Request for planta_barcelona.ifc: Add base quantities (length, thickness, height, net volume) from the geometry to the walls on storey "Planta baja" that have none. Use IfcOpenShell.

First a look at what the model holds.

```python
import ifcopenshell
import ifcopenshell.util.element
import ifcopenshell.util.unit

model = ifcopenshell.open("planta_barcelona.ifc")
print(model.schema)
for unit_type in ("LENGTHUNIT", "AREAUNIT", "VOLUMEUNIT"):
    print(unit_type, ifcopenshell.util.unit.calculate_unit_scale(model, unit_type))
storey = next(s for s in model.by_type("IfcBuildingStorey") if s.Name == "Planta baja")
walls = [e for e in ifcopenshell.util.element.get_decomposition(storey) if e.is_a("IfcWall")]
for e in sorted(walls, key=lambda e: e.id()):
    print(e.id(), e.is_a(), e.Name, list(ifcopenshell.util.element.get_psets(e, qtos_only=True)), sep=" | ")
```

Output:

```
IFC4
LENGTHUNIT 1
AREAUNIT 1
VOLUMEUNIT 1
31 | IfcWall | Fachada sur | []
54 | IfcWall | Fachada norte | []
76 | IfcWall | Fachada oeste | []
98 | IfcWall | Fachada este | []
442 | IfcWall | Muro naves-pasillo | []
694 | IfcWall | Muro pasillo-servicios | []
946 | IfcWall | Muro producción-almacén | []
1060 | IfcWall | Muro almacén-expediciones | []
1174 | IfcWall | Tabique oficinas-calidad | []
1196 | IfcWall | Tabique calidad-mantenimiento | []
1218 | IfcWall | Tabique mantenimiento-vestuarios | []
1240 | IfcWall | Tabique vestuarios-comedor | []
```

```python
import ifcopenshell
import ifcopenshell.api.pset
import ifcopenshell.geom
import ifcopenshell.util.element
import ifcopenshell.util.shape
import ifcopenshell.util.unit

model = ifcopenshell.open("planta_barcelona.ifc")
unit_scale = ifcopenshell.util.unit.calculate_unit_scale(model)
volume_scale = ifcopenshell.util.unit.calculate_unit_scale(model, "VOLUMEUNIT")
settings = ifcopenshell.geom.settings()

storey = next(s for s in model.by_type("IfcBuildingStorey") if s.Name == "Planta baja")
walls = [e for e in ifcopenshell.util.element.get_decomposition(storey) if e.is_a("IfcWall")]

for e in sorted(walls, key=lambda e: e.id()):
    if ifcopenshell.util.element.get_psets(e, qtos_only=True, should_inherit=False):
        continue
    # Geometry comes back in metres, in the element's own axes.
    shape = ifcopenshell.geom.create_shape(settings, e)
    values = {
        "Length": ifcopenshell.util.shape.get_x(shape.geometry) / unit_scale,
        "Width": ifcopenshell.util.shape.get_y(shape.geometry) / unit_scale,
        "Height": ifcopenshell.util.shape.get_z(shape.geometry) / unit_scale,
        "NetVolume": ifcopenshell.util.shape.get_volume(shape.geometry) / volume_scale,
    }
    qto = ifcopenshell.api.pset.add_qto(model, product=e, name="Qto_WallBaseQuantities")
    ifcopenshell.api.pset.edit_qto(model, qto=qto, properties=values)
    print(e.id(), {k: round(v, 3) for k, v in values.items()})

model.write("planta_barcelona-out.ifc")
```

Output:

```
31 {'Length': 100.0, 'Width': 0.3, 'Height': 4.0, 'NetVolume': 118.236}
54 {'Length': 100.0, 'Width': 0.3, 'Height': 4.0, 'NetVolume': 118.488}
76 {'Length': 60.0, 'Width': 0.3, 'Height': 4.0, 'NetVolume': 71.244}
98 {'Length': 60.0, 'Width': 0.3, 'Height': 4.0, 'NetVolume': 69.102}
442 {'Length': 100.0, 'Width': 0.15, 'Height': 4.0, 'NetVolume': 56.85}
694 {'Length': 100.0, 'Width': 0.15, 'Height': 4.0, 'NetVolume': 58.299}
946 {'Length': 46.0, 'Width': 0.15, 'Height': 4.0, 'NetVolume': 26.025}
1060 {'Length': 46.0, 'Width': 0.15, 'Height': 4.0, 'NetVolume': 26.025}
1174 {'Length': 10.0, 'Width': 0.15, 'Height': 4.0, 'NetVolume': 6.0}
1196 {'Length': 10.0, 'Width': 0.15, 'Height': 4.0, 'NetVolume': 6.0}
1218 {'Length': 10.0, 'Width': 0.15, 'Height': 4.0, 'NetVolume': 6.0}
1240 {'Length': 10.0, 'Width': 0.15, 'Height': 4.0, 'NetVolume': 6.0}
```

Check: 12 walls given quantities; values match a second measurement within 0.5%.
